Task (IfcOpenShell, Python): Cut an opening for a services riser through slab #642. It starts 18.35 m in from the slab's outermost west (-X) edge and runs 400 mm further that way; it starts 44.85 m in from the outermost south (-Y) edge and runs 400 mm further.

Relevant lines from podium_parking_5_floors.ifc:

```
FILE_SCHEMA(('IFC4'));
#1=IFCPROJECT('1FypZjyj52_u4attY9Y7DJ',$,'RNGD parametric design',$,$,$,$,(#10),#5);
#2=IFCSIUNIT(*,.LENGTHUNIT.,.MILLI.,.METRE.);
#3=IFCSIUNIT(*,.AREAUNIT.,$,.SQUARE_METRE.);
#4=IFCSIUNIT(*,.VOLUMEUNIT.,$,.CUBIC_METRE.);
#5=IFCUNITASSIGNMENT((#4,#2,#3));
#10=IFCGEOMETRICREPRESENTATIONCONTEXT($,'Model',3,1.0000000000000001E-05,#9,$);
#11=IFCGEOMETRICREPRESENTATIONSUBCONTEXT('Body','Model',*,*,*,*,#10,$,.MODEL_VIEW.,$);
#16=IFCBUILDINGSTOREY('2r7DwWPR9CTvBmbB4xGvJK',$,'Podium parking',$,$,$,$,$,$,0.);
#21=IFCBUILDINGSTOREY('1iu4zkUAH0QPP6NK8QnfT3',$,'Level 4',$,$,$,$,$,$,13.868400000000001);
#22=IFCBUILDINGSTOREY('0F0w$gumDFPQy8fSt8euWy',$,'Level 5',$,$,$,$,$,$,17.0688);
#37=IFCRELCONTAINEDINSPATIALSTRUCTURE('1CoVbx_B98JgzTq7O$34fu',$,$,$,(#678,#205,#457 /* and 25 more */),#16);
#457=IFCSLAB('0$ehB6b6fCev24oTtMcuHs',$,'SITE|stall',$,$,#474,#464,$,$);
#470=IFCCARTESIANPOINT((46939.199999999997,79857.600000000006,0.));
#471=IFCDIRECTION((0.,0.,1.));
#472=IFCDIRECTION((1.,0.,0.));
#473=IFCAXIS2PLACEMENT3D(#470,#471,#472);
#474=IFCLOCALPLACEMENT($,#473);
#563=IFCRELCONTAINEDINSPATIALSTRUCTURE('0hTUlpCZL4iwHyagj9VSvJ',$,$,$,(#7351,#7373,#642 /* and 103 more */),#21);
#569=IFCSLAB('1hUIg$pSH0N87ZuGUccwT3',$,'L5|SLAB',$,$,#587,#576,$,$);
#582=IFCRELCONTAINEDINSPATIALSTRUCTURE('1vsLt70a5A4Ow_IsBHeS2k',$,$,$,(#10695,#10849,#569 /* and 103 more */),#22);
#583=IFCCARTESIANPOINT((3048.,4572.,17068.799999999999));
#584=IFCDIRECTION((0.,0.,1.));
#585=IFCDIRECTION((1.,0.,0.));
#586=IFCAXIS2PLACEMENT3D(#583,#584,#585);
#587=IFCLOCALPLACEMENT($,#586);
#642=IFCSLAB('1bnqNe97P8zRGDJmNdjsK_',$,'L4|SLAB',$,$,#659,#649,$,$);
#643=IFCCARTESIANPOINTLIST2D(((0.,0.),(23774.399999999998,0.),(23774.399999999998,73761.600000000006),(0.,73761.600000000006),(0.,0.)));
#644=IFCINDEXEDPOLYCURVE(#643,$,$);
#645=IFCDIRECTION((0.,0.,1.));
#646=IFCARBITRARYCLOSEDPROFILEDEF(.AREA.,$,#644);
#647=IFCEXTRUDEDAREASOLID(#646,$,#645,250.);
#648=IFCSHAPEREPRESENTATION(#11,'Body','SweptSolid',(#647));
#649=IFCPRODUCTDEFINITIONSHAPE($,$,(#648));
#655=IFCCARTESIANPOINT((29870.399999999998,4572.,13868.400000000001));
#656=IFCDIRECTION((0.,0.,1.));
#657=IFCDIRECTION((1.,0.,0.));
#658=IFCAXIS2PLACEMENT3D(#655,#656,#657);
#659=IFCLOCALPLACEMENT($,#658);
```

```python
import numpy as np
import ifcopenshell
import ifcopenshell.api.feature
import ifcopenshell.api.geometry
import ifcopenshell.api.root
import ifcopenshell.geom
import ifcopenshell.util.placement
import ifcopenshell.util.representation
import ifcopenshell.util.shape
import ifcopenshell.util.unit

model = ifcopenshell.open("podium_parking_5_floors.ifc")
unit_scale = ifcopenshell.util.unit.calculate_unit_scale(model)
settings = ifcopenshell.geom.settings()


def volume(element):
    """Net volume in cubic metres, openings subtracted."""
    shape = ifcopenshell.geom.create_shape(settings, element)
    return ifcopenshell.util.shape.get_volume(shape.geometry)


slab = model.by_guid("1bnqNe97P8zRGDJmNdjsK_")
before = volume(slab)

# Extent in the slab's own axes, in metres. The edges named are its -X and -Y sides.
slab_shape = ifcopenshell.geom.create_shape(settings, slab)
vertices = ifcopenshell.util.shape.get_vertices(slab_shape.geometry)
x_min, y_min, bottom = vertices.min(axis=0)
top = vertices[:, 2].max()

opening = ifcopenshell.api.root.create_entity(model, ifc_class="IfcOpeningElement", name="Services riser opening", predefined_type="OPENING")
context = ifcopenshell.util.representation.get_context(model, "Model", "Body", "MODEL_VIEW")
width, depth = 0.4, 0.4
outline = [(0.0, 0.0), (width, 0.0), (width, depth), (0.0, depth), (0.0, 0.0)]
# Overshoot both faces by 50 mm so the cut is clean.
shape = ifcopenshell.api.geometry.add_slab_representation(
    model, context=context, depth=top - bottom + 0.1, polyline=outline
)
ifcopenshell.api.geometry.assign_representation(model, product=opening, representation=shape)

matrix = ifcopenshell.util.placement.get_local_placement(slab.ObjectPlacement)
matrix[:, 3] = matrix @ np.append(np.array([x_min + 18.35, y_min + 44.85, bottom - 0.05]) / unit_scale, 1.0)
ifcopenshell.api.geometry.edit_object_placement(model, product=opening, matrix=matrix, is_si=False)
ifcopenshell.api.feature.add_feature(model, feature=opening, element=slab)

after = volume(slab)

print(f"slab volume {before:.3f} -> {after:.3f} m3")

model.write("podium_parking_5_floors_v2.ifc")
```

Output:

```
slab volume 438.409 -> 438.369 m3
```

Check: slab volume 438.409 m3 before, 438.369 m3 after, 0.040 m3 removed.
